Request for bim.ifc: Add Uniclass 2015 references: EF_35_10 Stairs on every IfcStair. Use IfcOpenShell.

First a look at what the model holds.

```python
import ifcopenshell

model = ifcopenshell.open("bim.ifc")
print(model.schema)
print("classifications:", [c.Name for c in model.by_type("IfcClassification")])
for ifc_class in ("IfcDoor", "IfcRoof", "IfcStair", "IfcWall", "IfcWindow"):
    print(ifc_class, len(model.by_type(ifc_class)))
```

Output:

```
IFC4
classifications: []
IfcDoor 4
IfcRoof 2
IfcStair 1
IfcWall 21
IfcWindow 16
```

```python
import ifcopenshell
import ifcopenshell.api.classification

model = ifcopenshell.open("bim.ifc")

system = ifcopenshell.api.classification.add_classification(model, classification="Uniclass 2015")

codes = {
    "IfcStair": ("EF_35_10", "Stairs"),
}
for ifc_class, (code, name) in codes.items():
    products = model.by_type(ifc_class)
    ifcopenshell.api.classification.add_reference(
        model, products=products, classification=system, identification=code, name=name
    )
    print(code, len(products))

model.write("bim_edited.ifc")
```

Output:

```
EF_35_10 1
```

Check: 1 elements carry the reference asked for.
